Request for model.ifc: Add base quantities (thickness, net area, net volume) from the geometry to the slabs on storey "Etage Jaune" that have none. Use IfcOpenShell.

First a look at what the model holds.

```python
import ifcopenshell
import ifcopenshell.util.element
import ifcopenshell.util.unit

model = ifcopenshell.open("model.ifc")
print(model.schema)
for unit_type in ("LENGTHUNIT", "AREAUNIT", "VOLUMEUNIT"):
    print(unit_type, ifcopenshell.util.unit.calculate_unit_scale(model, unit_type))
storey = next(s for s in model.by_type("IfcBuildingStorey") if s.Name == "Etage Jaune")
slabs = [e for e in ifcopenshell.util.element.get_decomposition(storey) if e.is_a("IfcSlab")]
for e in sorted(slabs, key=lambda e: e.id()):
    print(e.id(), e.is_a(), e.Name, list(ifcopenshell.util.element.get_psets(e, qtos_only=True)), sep=" | ")
```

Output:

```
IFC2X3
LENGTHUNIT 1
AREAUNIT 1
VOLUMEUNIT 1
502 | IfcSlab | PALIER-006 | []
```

```python
import ifcopenshell
import ifcopenshell.api.pset
import ifcopenshell.geom
import ifcopenshell.util.element
import ifcopenshell.util.shape
import ifcopenshell.util.unit

model = ifcopenshell.open("model.ifc")
unit_scale = ifcopenshell.util.unit.calculate_unit_scale(model)
area_scale = ifcopenshell.util.unit.calculate_unit_scale(model, "AREAUNIT")
volume_scale = ifcopenshell.util.unit.calculate_unit_scale(model, "VOLUMEUNIT")
settings = ifcopenshell.geom.settings()

storey = next(s for s in model.by_type("IfcBuildingStorey") if s.Name == "Etage Jaune")
slabs = [e for e in ifcopenshell.util.element.get_decomposition(storey) if e.is_a("IfcSlab")]

for e in sorted(slabs, key=lambda e: e.id()):
    if ifcopenshell.util.element.get_psets(e, qtos_only=True, should_inherit=False):
        continue
    # Geometry comes back in metres, in the element's own axes.
    shape = ifcopenshell.geom.create_shape(settings, e)
    values = {
        "Width": ifcopenshell.util.shape.get_z(shape.geometry) / unit_scale,
        "NetArea": ifcopenshell.util.shape.get_footprint_area(shape.geometry) / area_scale,
        "NetVolume": ifcopenshell.util.shape.get_volume(shape.geometry) / volume_scale,
    }
    qto = ifcopenshell.api.pset.add_qto(model, product=e, name="BaseQuantities")
    ifcopenshell.api.pset.edit_qto(model, qto=qto, properties=values)
    print(e.id(), {k: round(v, 3) for k, v in values.items()})

model.write("model_updated.ifc")
```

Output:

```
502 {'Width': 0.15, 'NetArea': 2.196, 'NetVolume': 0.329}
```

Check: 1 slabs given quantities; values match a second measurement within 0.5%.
